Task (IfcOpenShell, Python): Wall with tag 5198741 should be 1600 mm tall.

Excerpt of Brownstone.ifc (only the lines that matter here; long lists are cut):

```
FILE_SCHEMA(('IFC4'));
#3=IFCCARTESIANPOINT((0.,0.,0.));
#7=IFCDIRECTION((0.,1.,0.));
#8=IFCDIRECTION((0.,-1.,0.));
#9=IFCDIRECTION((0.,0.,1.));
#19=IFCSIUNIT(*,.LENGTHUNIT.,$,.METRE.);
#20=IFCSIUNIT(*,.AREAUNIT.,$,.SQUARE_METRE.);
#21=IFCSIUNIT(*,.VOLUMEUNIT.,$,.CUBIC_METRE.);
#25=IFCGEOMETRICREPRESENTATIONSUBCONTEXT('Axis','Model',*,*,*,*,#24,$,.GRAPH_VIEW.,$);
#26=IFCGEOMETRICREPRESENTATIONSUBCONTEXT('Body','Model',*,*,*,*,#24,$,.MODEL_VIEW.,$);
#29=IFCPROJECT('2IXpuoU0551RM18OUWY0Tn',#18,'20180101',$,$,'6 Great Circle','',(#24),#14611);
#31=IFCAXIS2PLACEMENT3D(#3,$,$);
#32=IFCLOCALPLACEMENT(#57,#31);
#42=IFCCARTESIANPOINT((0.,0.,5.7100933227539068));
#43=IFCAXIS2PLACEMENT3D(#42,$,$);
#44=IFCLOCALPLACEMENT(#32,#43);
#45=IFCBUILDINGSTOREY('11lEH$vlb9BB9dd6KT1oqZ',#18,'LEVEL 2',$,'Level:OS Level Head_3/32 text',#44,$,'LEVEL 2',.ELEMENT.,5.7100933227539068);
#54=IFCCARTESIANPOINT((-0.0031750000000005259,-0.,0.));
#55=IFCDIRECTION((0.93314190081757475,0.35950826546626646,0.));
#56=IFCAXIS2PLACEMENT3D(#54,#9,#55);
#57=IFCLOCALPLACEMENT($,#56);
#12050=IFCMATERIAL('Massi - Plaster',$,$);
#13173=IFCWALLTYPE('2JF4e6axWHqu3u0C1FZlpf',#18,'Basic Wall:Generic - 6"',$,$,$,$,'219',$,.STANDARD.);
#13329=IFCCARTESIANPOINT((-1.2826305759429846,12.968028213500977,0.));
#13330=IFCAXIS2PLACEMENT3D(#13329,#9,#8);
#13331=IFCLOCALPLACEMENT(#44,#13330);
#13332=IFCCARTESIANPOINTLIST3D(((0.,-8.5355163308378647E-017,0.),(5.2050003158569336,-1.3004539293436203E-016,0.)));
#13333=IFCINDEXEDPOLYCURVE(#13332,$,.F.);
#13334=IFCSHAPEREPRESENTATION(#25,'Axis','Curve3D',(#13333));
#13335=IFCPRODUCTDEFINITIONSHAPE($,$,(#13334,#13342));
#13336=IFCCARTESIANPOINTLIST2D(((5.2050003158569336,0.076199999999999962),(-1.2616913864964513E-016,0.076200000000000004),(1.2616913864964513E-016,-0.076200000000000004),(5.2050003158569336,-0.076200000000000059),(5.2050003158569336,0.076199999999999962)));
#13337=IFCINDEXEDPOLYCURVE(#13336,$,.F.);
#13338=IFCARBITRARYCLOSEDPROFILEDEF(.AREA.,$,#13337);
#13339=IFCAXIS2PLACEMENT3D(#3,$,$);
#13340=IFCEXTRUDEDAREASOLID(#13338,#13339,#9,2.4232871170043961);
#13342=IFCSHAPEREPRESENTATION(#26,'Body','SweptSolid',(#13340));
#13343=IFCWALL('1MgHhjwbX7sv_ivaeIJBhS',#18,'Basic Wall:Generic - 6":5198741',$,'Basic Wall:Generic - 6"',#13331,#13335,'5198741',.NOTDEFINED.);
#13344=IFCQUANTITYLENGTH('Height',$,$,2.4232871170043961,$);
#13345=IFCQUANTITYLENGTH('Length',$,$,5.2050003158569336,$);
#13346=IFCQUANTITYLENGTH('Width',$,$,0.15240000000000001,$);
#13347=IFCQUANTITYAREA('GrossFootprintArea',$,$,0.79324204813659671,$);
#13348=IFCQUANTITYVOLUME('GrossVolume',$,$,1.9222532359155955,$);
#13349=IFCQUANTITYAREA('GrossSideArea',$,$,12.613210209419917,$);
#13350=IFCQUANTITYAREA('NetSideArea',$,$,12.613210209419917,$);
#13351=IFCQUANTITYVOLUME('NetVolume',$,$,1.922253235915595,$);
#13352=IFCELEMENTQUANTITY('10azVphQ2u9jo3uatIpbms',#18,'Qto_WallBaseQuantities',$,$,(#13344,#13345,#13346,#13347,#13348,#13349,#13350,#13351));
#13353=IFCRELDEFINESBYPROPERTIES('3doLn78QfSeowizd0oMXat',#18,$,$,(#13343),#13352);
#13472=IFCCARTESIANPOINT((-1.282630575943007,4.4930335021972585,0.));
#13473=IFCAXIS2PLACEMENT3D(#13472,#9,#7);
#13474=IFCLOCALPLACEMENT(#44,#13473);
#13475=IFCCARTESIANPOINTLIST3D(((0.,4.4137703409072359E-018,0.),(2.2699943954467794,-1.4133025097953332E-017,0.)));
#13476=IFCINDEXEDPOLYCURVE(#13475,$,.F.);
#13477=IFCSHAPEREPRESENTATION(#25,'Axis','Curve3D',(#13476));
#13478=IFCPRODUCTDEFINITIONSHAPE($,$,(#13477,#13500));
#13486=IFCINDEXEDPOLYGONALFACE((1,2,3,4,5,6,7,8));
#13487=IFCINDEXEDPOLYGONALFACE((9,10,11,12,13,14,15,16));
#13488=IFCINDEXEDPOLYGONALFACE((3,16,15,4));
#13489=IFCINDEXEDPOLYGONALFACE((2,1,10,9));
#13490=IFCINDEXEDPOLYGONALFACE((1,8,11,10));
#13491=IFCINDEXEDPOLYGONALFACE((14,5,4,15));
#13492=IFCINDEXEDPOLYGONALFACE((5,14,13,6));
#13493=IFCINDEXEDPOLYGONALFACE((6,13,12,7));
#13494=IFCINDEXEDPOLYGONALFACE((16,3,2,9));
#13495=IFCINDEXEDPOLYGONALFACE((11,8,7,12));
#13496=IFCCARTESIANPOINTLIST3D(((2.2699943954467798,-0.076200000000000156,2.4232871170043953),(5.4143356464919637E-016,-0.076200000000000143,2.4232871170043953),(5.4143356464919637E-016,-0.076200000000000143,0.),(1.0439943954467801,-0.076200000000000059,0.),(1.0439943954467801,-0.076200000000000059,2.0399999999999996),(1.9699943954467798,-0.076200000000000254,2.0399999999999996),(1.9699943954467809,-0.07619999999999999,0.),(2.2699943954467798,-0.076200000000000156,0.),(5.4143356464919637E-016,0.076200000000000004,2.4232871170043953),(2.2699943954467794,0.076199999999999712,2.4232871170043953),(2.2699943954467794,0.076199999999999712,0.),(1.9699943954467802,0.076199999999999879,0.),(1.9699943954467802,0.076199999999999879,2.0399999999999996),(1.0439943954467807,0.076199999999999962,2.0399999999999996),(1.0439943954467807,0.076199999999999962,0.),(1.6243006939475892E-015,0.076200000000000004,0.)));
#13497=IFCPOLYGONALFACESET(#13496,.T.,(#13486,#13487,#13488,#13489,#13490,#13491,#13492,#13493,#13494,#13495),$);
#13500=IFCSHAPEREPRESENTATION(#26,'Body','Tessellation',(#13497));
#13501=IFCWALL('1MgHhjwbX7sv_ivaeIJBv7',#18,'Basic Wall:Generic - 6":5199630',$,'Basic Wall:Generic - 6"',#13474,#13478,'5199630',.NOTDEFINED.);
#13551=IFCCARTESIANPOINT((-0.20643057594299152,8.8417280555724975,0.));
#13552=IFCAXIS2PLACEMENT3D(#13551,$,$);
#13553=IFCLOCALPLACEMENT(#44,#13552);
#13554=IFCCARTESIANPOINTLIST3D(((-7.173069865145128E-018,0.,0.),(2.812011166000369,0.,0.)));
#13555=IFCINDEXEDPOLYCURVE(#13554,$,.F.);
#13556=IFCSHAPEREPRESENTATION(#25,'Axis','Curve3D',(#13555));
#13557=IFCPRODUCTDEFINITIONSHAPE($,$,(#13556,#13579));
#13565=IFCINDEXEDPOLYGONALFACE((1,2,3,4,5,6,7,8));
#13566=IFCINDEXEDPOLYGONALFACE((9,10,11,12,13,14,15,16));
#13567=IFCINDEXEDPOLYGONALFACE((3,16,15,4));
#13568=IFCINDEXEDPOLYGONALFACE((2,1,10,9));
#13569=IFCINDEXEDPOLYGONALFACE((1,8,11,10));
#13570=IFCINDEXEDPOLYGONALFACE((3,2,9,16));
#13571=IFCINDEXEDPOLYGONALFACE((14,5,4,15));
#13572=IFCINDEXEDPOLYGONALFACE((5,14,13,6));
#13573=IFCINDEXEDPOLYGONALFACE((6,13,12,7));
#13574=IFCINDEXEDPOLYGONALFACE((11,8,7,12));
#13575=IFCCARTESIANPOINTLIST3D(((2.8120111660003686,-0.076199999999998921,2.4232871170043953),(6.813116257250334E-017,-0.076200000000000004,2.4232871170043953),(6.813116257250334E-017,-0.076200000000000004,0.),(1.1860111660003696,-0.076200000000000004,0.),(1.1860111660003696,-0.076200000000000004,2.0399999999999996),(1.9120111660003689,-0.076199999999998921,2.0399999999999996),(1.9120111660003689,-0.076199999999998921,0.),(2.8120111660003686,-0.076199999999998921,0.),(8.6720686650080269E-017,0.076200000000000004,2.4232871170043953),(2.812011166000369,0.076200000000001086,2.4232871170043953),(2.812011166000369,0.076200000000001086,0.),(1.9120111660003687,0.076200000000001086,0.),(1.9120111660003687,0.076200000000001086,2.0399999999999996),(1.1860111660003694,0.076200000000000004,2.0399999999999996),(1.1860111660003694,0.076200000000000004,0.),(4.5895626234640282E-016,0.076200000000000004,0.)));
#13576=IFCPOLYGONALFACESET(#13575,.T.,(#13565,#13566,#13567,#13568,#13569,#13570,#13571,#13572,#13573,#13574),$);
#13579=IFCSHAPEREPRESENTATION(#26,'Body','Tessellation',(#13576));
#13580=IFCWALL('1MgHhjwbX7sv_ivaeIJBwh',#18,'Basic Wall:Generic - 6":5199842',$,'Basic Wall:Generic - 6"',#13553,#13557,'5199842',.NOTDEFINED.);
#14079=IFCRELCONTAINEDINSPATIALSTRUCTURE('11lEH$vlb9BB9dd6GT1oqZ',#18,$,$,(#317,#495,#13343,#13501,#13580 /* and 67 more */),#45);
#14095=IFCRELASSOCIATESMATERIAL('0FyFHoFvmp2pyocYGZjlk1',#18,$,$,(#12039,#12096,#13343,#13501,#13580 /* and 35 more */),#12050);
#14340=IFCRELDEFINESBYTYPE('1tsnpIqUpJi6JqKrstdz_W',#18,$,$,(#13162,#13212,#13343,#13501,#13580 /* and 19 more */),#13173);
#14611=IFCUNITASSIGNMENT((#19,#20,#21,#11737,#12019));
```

```python
import ifcopenshell
import ifcopenshell.api.pset
import ifcopenshell.geom
import ifcopenshell.util.element
import ifcopenshell.util.representation
import ifcopenshell.util.shape
import ifcopenshell.util.unit

model = ifcopenshell.open("Brownstone.ifc")
unit_scale = ifcopenshell.util.unit.calculate_unit_scale(model)
area_scale = ifcopenshell.util.unit.calculate_unit_scale(model, "AREAUNIT")
volume_scale = ifcopenshell.util.unit.calculate_unit_scale(model, "VOLUMEUNIT")
settings = ifcopenshell.geom.settings()


def volume(element):
    """Net volume in cubic metres, openings subtracted."""
    shape = ifcopenshell.geom.create_shape(settings, element)
    return ifcopenshell.util.shape.get_volume(shape.geometry)


wall = model.by_guid("1MgHhjwbX7sv_ivaeIJBhS")
before = volume(wall)

body = ifcopenshell.util.representation.get_representation(wall, "Model", "Body")
solid = body.Items[0]
old_height = solid.Depth
solid.Depth = 1.6 / unit_scale
after = volume(wall)
thickness = 0.1524  # wall thickness in metres

# Update the stored height, areas and volumes.
qto = model.by_id(ifcopenshell.util.element.get_pset(wall, "Qto_WallBaseQuantities", should_inherit=False)["id"])
ifcopenshell.api.pset.edit_qto(model, qto=qto, properties={
    "Height": solid.Depth,
    "GrossVolume": ifcopenshell.util.element.get_pset(wall, "Qto_WallBaseQuantities", "GrossVolume") * solid.Depth / old_height,
    "GrossSideArea": ifcopenshell.util.element.get_pset(wall, "Qto_WallBaseQuantities", "GrossSideArea") * solid.Depth / old_height,
    "NetSideArea": after / thickness / area_scale,
    "NetVolume": after / volume_scale,
})

print(f"height {old_height:g} -> {solid.Depth:g}, volume {before:.3f} -> {after:.3f} m3")

model.write("Brownstone_edited.ifc")
```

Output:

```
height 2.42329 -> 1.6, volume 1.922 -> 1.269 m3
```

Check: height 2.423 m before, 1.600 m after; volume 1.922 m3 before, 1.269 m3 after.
